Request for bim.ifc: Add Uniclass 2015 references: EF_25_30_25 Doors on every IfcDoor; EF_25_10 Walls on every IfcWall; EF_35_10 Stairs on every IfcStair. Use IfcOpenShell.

First a look at what the model holds.

```python
import ifcopenshell

model = ifcopenshell.open("bim.ifc")
print(model.schema)
print("classifications:", [c.Name for c in model.by_type("IfcClassification")])
for ifc_class in ("IfcDoor", "IfcRoof", "IfcStair", "IfcWall", "IfcWindow"):
    print(ifc_class, len(model.by_type(ifc_class)))
```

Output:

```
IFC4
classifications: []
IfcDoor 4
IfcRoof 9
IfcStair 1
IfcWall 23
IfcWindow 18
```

```python
import ifcopenshell
import ifcopenshell.api.classification

model = ifcopenshell.open("bim.ifc")

system = ifcopenshell.api.classification.add_classification(model, classification="Uniclass 2015")

codes = {
    "IfcDoor": ("EF_25_30_25", "Doors"),
    "IfcWall": ("EF_25_10", "Walls"),
    "IfcStair": ("EF_35_10", "Stairs"),
}
for ifc_class, (code, name) in codes.items():
    products = model.by_type(ifc_class)
    ifcopenshell.api.classification.add_reference(
        model, products=products, classification=system, identification=code, name=name
    )
    print(code, len(products))

model.write("bim_edited.ifc")
```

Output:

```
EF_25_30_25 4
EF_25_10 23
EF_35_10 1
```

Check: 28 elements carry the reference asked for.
